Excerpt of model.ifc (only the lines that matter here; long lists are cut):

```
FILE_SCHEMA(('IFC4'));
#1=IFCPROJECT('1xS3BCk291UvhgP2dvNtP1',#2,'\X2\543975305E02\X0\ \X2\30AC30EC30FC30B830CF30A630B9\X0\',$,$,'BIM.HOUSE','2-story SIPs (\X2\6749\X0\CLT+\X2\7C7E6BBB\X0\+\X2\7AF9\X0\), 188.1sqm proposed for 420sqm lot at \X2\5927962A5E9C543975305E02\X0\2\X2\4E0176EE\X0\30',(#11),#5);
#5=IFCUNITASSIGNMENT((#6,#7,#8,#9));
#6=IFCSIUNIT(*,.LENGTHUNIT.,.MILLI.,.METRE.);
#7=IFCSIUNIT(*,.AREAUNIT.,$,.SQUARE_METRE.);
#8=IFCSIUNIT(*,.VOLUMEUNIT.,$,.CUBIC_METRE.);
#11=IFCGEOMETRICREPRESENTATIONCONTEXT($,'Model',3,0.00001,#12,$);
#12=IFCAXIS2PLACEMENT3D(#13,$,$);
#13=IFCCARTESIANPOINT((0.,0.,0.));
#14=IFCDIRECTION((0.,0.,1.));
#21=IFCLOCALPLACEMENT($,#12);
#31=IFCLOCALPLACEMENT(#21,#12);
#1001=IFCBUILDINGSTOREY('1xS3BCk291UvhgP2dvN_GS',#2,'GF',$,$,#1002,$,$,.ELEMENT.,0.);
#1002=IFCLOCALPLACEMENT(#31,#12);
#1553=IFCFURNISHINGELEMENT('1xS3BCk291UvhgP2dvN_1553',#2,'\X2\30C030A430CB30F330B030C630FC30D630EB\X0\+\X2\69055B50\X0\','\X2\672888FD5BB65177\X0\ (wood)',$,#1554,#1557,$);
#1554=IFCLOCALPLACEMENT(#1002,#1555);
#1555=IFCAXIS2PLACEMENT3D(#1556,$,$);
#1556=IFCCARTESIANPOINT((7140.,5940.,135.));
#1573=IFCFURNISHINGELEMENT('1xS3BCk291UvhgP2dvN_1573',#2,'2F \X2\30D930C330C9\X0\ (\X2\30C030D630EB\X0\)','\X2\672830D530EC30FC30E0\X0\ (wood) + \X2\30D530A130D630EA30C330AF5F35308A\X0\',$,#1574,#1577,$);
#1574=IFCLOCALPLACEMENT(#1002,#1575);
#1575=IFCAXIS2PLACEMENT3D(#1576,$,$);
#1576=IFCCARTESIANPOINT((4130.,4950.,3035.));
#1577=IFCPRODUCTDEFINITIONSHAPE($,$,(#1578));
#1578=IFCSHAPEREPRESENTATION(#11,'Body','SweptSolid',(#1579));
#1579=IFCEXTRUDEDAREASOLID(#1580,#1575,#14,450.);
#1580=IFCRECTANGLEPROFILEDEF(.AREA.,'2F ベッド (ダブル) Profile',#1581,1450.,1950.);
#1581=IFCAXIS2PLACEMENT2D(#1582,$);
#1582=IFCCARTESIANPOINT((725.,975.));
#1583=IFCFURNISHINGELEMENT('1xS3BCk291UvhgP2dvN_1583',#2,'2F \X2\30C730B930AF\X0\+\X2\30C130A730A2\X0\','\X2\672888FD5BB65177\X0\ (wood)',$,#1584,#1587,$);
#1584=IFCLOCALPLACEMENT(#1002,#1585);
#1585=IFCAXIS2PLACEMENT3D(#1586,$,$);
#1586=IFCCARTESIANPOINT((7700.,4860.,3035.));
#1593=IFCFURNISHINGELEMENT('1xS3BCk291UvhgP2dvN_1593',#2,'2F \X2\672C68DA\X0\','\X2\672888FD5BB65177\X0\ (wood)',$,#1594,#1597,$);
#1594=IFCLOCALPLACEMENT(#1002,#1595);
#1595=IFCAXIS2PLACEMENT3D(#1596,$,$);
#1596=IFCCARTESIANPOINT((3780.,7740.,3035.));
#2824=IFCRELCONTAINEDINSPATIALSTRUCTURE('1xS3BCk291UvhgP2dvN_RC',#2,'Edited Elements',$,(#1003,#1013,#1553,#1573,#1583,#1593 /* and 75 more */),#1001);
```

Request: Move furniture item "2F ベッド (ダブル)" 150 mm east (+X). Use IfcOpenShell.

```python
import ifcopenshell
import ifcopenshell.api.geometry
import ifcopenshell.util.placement

model = ifcopenshell.open("model.ifc")

item = model.by_guid("1xS3BCk291UvhgP2dvN_1573")
matrix = ifcopenshell.util.placement.get_local_placement(item.ObjectPlacement)
matrix[0, 3] += 150.0
ifcopenshell.api.geometry.edit_object_placement(model, product=item, matrix=matrix, is_si=False)

print(ifcopenshell.util.placement.get_local_placement(item.ObjectPlacement).round(3) + 0.0)

model.write("model_edited.ifc")
```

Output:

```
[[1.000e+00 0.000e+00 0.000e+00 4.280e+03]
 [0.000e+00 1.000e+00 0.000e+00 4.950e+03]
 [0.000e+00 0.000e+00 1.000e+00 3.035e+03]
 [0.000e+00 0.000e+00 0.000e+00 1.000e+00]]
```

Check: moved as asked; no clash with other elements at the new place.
